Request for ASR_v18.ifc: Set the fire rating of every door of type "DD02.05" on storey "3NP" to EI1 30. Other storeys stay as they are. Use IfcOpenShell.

First a look at what the model holds.

```python
import ifcopenshell
import ifcopenshell.util.element

model = ifcopenshell.open("ASR_v18.ifc")
print(model.schema)
storey = next(s for s in model.by_type("IfcBuildingStorey") if s.Name == "3NP")
doors = [e for e in ifcopenshell.util.element.get_decomposition(storey) if e.is_a("IfcDoor")]
seen = {}
for e in doors:
    element_type = ifcopenshell.util.element.get_type(e)
    key = (element_type.Name if element_type != e and element_type else None, ifcopenshell.util.element.get_pset(e, "Pset_DoorCommon", "FireRating"))
    seen[key] = seen.get(key, 0) + 1
for (name, value), count in sorted(seen.items(), key=str):
    print(count, "x", name, "|", value)
```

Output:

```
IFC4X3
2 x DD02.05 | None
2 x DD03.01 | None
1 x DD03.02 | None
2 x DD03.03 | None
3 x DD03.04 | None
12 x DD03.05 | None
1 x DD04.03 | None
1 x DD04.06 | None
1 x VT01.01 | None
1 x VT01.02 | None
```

```python
import ifcopenshell
import ifcopenshell.api.pset
import ifcopenshell.util.element

model = ifcopenshell.open("ASR_v18.ifc")

storey = next(s for s in model.by_type("IfcBuildingStorey") if s.Name == "3NP")
doors = [e for e in ifcopenshell.util.element.get_decomposition(storey) if e.is_a("IfcDoor")]

count = 0
for e in doors:
    element_type = ifcopenshell.util.element.get_type(e)
    if element_type in (None, e) or element_type.Name != "DD02.05":
        continue
    # add_pset returns the element's existing set when there is one.
    pset = ifcopenshell.api.pset.add_pset(model, product=e, name="Pset_DoorCommon")
    ifcopenshell.api.pset.edit_pset(model, pset=pset, properties={"FireRating": "EI1 30"})
    count += 1

print(count, "doors updated")

model.write("ASR_v18_updated.ifc")
```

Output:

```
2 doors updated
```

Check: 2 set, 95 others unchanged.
